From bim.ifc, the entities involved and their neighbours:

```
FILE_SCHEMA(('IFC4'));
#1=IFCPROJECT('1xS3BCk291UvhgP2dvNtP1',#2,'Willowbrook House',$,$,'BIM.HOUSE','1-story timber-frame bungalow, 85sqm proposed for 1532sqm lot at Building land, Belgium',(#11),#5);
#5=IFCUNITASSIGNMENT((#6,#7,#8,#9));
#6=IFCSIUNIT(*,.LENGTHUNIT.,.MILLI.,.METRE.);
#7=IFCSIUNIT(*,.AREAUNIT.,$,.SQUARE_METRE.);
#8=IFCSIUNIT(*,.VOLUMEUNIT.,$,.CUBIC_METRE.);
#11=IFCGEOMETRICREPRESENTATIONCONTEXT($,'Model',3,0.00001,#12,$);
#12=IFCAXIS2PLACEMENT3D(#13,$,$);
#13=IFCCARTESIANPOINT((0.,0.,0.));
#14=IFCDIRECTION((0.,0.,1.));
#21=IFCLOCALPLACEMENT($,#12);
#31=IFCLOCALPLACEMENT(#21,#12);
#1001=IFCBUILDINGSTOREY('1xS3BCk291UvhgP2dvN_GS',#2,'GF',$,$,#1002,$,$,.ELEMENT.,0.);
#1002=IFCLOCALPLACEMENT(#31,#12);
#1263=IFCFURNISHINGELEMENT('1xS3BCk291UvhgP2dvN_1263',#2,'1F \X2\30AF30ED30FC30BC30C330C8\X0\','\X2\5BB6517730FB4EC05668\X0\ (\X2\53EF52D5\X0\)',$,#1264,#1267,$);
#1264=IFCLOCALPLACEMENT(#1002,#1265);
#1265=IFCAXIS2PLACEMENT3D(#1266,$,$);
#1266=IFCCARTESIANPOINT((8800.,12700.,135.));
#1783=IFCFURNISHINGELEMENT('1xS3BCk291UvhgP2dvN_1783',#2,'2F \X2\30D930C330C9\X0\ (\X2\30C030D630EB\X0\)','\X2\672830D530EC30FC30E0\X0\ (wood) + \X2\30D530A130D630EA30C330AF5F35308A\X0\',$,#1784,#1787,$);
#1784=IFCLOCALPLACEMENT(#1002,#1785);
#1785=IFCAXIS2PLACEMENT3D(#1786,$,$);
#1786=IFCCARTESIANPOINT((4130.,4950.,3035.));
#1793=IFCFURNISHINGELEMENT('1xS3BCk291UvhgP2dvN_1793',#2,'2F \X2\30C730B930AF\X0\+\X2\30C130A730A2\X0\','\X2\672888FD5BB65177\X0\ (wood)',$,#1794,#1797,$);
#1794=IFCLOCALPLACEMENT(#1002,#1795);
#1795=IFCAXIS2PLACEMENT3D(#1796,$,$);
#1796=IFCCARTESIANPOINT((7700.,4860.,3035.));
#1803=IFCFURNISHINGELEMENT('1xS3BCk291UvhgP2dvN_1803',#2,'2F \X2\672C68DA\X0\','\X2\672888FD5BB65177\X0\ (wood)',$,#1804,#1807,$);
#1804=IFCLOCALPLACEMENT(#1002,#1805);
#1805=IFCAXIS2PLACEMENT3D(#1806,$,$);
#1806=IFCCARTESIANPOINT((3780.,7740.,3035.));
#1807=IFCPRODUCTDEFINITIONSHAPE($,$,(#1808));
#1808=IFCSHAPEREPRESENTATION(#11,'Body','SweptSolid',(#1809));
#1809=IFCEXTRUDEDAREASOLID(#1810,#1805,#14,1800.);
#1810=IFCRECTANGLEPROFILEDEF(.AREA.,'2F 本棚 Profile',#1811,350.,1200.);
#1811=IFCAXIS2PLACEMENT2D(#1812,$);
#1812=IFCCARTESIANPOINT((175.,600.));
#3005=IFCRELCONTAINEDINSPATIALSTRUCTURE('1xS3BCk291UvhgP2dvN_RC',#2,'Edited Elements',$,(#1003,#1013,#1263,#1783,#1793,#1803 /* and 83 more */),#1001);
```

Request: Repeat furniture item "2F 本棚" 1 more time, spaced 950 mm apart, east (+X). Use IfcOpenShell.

```python
import numpy as np
import ifcopenshell
import ifcopenshell.api.geometry
import ifcopenshell.api.root
import ifcopenshell.util.element
import ifcopenshell.util.placement

model = ifcopenshell.open("bim.ifc")


def reuse_history(source, copy):
    """copy_class also copies each property set's owner history, people and application; keep the originals."""
    for rel in copy.IsDefinedBy:
        if rel.is_a("IfcRelDefinesByProperties") and (history := rel.RelatingPropertyDefinition.OwnerHistory):
            rel.RelatingPropertyDefinition.OwnerHistory = source.OwnerHistory
            ifcopenshell.util.element.remove_deep2(model, history)


source = model.by_guid("1xS3BCk291UvhgP2dvN_1803")
base = ifcopenshell.util.placement.get_local_placement(source.ObjectPlacement)
step = np.array([1.0, 0.0, 0.0]) * 950.0

for i in range(1, 2):
    copy = ifcopenshell.api.root.copy_class(model, product=source)
    copy.Representation = ifcopenshell.util.element.copy_deep(
        model, source.Representation, exclude=["IfcGeometricRepresentationContext", "IfcRepresentationMap"]
    )
    reuse_history(source, copy)
    matrix = base.copy()
    matrix[:3, 3] += i * step
    print("added at", matrix[:3, 3].round(3) + 0.0)
    ifcopenshell.api.geometry.edit_object_placement(model, product=copy, matrix=matrix, is_si=False)

model.write("bim_rev.ifc")
```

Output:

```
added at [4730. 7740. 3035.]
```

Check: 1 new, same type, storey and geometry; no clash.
